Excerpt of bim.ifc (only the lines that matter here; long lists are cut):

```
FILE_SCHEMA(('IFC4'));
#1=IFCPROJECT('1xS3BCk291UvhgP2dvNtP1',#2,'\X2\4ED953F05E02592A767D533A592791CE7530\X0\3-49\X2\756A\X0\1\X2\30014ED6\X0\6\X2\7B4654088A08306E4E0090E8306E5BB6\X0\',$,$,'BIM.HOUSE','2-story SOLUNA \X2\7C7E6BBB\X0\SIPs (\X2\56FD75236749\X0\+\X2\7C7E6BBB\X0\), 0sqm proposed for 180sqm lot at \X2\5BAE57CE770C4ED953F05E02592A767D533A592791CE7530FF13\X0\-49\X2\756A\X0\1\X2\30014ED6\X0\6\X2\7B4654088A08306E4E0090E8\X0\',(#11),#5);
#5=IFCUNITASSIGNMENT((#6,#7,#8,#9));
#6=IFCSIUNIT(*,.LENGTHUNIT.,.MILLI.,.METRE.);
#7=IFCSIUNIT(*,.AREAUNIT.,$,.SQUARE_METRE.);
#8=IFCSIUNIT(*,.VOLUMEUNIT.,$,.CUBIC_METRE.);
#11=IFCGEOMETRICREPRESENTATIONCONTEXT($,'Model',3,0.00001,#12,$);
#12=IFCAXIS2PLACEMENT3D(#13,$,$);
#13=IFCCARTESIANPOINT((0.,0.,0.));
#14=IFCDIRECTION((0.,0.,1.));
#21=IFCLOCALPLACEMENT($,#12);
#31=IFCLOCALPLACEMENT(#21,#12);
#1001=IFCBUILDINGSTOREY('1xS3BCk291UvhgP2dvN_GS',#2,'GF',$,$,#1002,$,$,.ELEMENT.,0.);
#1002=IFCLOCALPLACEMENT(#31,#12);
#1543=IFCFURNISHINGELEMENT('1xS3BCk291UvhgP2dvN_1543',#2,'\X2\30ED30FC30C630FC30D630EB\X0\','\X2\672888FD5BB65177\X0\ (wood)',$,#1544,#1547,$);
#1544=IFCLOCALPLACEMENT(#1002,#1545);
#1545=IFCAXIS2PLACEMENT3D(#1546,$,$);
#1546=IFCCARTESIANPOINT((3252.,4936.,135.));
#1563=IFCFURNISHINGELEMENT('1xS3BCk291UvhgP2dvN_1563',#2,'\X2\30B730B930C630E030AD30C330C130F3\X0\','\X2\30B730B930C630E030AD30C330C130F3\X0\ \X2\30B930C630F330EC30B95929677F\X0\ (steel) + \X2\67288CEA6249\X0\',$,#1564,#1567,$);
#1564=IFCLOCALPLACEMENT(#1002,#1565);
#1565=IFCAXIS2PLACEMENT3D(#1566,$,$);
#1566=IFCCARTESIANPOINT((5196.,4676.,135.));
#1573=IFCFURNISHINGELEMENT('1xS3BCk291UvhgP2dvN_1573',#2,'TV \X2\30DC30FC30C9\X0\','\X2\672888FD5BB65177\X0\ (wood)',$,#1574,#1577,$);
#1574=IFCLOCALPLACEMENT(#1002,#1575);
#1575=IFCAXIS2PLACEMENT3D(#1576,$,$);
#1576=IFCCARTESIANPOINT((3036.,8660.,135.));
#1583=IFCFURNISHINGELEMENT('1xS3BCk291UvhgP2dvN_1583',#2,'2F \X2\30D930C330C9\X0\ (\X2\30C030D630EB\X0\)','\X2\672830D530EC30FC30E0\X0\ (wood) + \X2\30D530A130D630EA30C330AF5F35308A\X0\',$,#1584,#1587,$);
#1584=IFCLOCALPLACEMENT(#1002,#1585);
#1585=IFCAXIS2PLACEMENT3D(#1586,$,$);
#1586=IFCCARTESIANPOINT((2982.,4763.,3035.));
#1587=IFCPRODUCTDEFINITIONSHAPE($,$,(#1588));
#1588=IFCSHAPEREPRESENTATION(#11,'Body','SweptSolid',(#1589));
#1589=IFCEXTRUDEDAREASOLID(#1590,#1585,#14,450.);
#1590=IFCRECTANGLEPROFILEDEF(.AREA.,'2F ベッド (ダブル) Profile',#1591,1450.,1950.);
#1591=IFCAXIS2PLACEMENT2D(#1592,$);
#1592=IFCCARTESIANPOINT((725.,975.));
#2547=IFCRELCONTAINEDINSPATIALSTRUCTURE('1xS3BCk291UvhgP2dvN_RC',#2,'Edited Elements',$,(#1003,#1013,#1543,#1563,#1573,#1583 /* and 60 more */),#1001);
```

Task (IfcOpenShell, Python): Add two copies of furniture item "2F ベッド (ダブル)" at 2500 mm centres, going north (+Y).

```python
import numpy as np
import ifcopenshell
import ifcopenshell.api.geometry
import ifcopenshell.api.root
import ifcopenshell.util.element
import ifcopenshell.util.placement

model = ifcopenshell.open("bim.ifc")


def reuse_history(source, copy):
    """copy_class also copies each property set's owner history, people and application; keep the originals."""
    for rel in copy.IsDefinedBy:
        if rel.is_a("IfcRelDefinesByProperties") and (history := rel.RelatingPropertyDefinition.OwnerHistory):
            rel.RelatingPropertyDefinition.OwnerHistory = source.OwnerHistory
            ifcopenshell.util.element.remove_deep2(model, history)


source = model.by_id(1583)
base = ifcopenshell.util.placement.get_local_placement(source.ObjectPlacement)
step = np.array([0.0, 1.0, 0.0]) * 2500.0

for i in range(1, 3):
    copy = ifcopenshell.api.root.copy_class(model, product=source)
    copy.Representation = ifcopenshell.util.element.copy_deep(
        model, source.Representation, exclude=["IfcGeometricRepresentationContext", "IfcRepresentationMap"]
    )
    reuse_history(source, copy)
    matrix = base.copy()
    matrix[:3, 3] += i * step
    print("added at", matrix[:3, 3].round(3) + 0.0)
    ifcopenshell.api.geometry.edit_object_placement(model, product=copy, matrix=matrix, is_si=False)

model.write("bim_updated.ifc")
```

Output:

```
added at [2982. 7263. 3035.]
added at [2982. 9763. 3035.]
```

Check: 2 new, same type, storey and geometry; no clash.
